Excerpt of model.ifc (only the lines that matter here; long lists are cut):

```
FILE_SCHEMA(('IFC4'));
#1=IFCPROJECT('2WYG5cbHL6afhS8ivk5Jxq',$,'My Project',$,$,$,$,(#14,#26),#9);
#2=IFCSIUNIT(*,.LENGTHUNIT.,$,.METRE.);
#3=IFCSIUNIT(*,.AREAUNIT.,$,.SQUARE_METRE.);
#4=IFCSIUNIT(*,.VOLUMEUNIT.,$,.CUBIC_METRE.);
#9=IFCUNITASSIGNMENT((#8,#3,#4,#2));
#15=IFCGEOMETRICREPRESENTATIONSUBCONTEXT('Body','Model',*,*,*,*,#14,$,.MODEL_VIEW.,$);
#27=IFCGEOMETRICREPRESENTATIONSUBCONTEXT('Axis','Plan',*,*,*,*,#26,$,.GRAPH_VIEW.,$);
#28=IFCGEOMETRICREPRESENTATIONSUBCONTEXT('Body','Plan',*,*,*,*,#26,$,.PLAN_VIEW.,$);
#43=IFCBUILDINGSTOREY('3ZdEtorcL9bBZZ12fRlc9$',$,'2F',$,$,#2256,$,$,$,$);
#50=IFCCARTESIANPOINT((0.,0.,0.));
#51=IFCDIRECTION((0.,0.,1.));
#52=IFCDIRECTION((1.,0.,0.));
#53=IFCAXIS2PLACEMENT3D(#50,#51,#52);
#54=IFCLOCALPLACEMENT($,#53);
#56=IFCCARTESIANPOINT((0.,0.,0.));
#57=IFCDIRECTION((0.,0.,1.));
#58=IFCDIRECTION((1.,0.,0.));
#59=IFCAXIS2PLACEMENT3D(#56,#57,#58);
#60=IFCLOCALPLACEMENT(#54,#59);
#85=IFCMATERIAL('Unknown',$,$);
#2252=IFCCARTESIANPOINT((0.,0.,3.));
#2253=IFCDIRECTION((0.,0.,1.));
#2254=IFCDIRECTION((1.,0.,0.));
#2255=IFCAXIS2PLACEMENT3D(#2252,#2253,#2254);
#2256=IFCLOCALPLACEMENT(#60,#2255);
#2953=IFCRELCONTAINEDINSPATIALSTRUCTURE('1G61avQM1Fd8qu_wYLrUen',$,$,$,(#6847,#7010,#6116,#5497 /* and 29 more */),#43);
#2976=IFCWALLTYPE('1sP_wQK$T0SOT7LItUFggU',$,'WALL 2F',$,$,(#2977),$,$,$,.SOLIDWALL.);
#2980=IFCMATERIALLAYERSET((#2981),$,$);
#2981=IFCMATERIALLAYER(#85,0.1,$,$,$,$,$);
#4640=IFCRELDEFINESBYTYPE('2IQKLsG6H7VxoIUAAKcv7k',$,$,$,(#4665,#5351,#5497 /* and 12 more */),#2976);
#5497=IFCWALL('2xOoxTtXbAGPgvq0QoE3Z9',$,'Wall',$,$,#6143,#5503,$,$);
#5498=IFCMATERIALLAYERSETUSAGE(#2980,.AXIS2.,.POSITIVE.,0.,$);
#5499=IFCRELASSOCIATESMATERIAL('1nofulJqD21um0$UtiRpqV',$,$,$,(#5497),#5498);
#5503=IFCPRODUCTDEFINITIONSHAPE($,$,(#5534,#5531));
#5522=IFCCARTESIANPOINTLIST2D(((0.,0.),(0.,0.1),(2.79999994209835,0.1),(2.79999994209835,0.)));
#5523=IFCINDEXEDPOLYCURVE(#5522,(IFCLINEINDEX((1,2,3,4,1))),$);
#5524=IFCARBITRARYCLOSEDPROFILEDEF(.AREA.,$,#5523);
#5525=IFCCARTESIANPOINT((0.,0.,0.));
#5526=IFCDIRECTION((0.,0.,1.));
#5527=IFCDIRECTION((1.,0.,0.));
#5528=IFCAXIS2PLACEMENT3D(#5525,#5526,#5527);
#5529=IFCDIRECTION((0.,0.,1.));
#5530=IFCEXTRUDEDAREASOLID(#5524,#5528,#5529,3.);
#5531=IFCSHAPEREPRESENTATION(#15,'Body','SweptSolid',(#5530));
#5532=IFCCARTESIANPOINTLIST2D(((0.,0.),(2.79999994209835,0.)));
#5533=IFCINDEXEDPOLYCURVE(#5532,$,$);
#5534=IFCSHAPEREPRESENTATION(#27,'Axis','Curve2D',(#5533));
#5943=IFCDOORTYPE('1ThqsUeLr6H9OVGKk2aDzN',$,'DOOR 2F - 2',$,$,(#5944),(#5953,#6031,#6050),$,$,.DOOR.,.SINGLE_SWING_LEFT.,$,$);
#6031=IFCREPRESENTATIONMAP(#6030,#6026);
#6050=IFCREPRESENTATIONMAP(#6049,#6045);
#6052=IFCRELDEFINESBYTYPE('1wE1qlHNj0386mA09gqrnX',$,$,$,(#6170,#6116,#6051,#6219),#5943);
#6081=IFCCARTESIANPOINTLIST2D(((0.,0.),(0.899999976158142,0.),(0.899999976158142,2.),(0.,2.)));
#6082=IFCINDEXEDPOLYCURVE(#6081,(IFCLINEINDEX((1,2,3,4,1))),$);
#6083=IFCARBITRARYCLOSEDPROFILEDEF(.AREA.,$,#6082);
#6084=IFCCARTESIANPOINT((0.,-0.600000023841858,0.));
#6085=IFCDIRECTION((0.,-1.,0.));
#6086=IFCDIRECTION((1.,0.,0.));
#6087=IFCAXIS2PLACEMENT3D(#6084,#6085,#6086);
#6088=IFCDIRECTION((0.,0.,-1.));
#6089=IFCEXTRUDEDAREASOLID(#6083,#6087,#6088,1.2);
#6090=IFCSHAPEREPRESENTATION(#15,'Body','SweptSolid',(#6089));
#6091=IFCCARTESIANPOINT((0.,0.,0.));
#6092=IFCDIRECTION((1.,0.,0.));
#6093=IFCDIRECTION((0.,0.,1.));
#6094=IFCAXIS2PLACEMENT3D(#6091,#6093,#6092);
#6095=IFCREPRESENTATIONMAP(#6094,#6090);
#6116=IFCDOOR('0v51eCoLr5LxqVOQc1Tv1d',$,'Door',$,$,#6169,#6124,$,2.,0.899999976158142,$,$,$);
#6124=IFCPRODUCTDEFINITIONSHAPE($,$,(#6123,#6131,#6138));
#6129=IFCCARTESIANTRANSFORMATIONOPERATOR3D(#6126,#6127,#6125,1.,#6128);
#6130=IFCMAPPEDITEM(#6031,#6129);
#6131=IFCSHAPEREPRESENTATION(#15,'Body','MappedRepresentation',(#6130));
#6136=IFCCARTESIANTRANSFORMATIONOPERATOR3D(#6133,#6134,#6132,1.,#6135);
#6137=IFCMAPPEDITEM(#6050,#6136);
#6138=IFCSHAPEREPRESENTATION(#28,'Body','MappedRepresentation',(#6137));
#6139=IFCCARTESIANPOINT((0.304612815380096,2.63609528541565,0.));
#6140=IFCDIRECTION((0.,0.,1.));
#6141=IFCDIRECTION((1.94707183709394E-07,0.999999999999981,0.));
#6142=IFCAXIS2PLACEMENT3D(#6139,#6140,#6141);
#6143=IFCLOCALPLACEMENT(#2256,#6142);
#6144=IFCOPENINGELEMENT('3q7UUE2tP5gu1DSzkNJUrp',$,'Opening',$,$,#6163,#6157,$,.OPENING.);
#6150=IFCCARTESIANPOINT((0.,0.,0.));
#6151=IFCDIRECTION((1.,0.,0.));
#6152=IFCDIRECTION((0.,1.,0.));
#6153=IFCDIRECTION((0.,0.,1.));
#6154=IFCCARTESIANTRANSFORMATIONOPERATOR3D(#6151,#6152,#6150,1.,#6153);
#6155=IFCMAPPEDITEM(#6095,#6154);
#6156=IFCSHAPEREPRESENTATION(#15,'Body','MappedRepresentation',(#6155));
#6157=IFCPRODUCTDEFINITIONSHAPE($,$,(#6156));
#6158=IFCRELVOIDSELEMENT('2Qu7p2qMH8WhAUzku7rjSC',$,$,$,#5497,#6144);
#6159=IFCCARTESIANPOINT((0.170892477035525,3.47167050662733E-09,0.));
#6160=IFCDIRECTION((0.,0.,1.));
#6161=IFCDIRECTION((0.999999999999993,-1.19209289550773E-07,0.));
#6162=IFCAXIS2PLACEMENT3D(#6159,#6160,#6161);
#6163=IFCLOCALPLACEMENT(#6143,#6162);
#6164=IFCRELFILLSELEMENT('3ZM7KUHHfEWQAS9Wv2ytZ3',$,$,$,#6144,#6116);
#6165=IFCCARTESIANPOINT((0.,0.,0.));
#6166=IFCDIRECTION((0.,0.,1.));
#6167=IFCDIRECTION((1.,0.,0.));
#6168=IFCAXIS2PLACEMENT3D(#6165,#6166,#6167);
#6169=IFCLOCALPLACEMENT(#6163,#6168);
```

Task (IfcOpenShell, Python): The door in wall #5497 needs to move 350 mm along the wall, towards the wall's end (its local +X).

```python
import ifcopenshell
import ifcopenshell.api.geometry
import ifcopenshell.util.placement
import ifcopenshell.util.unit

model = ifcopenshell.open("model.ifc")
unit_scale = ifcopenshell.util.unit.calculate_unit_scale(model)

door = model.by_guid("0v51eCoLr5LxqVOQc1Tv1d")
opening = door.FillsVoids[0].RelatingOpeningElement
wall = opening.VoidsElements[0].RelatingBuildingElement

wall_matrix = ifcopenshell.util.placement.get_local_placement(wall.ObjectPlacement)
shift = wall_matrix[:3, 0] * 0.35 / unit_scale
before = ifcopenshell.util.placement.get_local_placement(door.ObjectPlacement)[:3, 3].copy()

# The door is placed relative to its opening, so it follows when the opening moves.
matrix = ifcopenshell.util.placement.get_local_placement(opening.ObjectPlacement)
matrix[:3, 3] += shift
ifcopenshell.api.geometry.edit_object_placement(
    model, product=opening, matrix=matrix, is_si=False, should_transform_children=True
)

after = ifcopenshell.util.placement.get_local_placement(door.ObjectPlacement)[:3, 3]
print("door moved by", (after - before).round(3) + 0.0)

model.write("model-out.ifc")
```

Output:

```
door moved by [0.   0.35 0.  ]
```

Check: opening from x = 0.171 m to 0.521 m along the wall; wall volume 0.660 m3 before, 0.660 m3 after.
